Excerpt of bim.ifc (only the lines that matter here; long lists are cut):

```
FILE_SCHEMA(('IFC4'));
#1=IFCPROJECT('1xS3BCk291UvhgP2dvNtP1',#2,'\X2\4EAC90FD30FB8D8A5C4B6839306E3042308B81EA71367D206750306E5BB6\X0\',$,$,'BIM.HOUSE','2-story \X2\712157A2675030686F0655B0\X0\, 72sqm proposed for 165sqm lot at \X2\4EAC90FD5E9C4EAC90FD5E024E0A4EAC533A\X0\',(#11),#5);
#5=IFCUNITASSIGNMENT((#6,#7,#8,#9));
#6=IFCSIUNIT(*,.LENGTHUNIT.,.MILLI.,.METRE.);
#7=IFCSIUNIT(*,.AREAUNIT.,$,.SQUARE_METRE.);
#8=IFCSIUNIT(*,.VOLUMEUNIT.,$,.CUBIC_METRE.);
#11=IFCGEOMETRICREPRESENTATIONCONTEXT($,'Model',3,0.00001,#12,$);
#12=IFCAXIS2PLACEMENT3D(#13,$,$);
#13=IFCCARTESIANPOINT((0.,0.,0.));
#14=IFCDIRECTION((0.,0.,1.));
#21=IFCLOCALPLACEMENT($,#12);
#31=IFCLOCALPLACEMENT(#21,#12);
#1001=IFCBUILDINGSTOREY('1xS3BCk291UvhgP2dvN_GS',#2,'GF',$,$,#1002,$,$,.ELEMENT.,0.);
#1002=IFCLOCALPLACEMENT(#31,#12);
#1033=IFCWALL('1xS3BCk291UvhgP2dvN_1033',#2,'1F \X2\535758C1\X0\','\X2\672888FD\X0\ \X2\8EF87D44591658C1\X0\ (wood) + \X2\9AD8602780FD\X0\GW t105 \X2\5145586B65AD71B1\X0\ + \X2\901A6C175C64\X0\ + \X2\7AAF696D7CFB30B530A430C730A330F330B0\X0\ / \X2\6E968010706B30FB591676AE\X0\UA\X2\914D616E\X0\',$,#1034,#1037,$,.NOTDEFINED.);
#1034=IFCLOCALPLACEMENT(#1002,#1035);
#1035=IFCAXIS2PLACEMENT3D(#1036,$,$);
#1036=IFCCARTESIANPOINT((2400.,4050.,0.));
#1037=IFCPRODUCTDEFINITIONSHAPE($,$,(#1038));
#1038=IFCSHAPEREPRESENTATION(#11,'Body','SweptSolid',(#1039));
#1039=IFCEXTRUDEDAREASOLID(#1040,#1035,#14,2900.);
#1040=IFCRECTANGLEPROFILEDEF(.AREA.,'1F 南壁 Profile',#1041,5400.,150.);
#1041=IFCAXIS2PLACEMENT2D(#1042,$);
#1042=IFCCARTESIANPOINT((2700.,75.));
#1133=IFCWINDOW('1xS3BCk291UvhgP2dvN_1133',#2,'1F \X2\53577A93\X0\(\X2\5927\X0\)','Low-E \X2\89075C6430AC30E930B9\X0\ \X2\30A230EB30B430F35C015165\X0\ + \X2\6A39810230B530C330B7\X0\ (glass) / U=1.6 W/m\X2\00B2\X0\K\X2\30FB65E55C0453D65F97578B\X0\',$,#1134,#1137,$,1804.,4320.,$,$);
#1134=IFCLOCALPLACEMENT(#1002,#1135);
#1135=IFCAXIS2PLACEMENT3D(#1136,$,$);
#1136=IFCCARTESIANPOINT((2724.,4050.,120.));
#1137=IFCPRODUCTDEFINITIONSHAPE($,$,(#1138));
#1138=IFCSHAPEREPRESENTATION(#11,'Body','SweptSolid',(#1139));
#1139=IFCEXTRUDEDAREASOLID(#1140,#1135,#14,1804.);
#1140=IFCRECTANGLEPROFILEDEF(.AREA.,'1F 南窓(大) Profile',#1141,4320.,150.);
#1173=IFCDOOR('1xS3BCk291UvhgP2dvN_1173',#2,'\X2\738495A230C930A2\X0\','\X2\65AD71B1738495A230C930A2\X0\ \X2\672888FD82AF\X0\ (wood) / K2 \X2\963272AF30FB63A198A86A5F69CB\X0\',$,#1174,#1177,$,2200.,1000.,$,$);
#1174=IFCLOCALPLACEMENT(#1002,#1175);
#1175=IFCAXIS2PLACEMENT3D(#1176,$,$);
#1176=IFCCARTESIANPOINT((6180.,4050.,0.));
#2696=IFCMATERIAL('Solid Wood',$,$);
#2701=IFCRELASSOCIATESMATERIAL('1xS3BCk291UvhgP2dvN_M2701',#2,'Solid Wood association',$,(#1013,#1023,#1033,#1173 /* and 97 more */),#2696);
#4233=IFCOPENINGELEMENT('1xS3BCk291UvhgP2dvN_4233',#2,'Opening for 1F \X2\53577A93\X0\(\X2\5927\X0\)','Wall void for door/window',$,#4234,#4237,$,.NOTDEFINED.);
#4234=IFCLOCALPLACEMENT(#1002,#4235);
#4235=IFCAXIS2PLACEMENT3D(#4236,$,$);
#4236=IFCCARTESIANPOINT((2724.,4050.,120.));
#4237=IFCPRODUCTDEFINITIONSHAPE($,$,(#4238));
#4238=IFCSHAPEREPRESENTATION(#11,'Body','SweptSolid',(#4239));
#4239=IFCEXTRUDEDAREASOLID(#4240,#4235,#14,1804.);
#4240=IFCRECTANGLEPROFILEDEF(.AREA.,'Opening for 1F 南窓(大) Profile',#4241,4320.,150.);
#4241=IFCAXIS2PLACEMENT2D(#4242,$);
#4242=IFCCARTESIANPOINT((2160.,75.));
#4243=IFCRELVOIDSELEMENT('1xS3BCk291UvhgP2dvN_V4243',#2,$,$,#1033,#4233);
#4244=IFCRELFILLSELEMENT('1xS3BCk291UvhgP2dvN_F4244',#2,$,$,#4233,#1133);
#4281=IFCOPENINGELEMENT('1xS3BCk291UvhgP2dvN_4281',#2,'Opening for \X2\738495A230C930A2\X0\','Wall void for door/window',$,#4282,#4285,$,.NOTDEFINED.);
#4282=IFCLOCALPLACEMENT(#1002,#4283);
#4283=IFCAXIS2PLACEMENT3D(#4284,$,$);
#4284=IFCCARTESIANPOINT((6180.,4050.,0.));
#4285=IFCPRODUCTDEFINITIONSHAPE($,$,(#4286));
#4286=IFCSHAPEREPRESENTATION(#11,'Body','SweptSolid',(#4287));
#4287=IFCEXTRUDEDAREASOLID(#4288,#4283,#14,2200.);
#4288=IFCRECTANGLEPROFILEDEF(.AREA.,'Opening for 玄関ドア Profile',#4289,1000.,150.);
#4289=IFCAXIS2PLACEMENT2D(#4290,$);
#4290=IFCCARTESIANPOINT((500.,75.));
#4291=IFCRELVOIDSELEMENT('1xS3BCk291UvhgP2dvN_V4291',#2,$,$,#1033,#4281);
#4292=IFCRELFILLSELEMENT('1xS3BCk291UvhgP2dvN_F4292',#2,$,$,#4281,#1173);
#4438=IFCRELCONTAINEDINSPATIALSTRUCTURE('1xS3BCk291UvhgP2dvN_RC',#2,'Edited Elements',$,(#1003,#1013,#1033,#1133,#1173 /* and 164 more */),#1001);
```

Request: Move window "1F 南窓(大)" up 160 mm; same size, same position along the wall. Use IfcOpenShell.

```python
import numpy as np
import ifcopenshell
import ifcopenshell.api.geometry
import ifcopenshell.util.placement
import ifcopenshell.util.unit

model = ifcopenshell.open("bim.ifc")
unit_scale = ifcopenshell.util.unit.calculate_unit_scale(model)

window = model.by_guid("1xS3BCk291UvhgP2dvN_1133")
opening = window.FillsVoids[0].RelatingOpeningElement
dz = 160.0

shift = np.array([0.0, 0.0, dz])
# The window is not placed relative to its opening, so move both.
for product in (opening, window):
    matrix = ifcopenshell.util.placement.get_local_placement(product.ObjectPlacement)
    matrix[:3, 3] += shift
    ifcopenshell.api.geometry.edit_object_placement(model, product=product, matrix=matrix, is_si=False)

print(f"moved by {dz * unit_scale:+.3f} m")

model.write("bim_edited.ifc")
```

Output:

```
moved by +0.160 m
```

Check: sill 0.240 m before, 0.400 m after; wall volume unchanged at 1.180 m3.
